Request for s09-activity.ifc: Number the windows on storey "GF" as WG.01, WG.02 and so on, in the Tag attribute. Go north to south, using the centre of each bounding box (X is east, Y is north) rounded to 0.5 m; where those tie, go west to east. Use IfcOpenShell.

First a look at what the model holds.

```python
import ifcopenshell
import ifcopenshell.util.element
import ifcopenshell.util.placement

model = ifcopenshell.open("s09-activity.ifc")
print(model.schema)
storey = next(s for s in model.by_type("IfcBuildingStorey") if s.Name == "GF")
windows = [e for e in ifcopenshell.util.element.get_decomposition(storey) if e.is_a("IfcWindow")]
for e in sorted(windows, key=lambda e: e.id()):
    origin = ifcopenshell.util.placement.get_local_placement(e.ObjectPlacement)[:3, 3]
    print(e.id(), e.Tag, e.Name, origin.round(2) + 0.0, sep=" | ")
```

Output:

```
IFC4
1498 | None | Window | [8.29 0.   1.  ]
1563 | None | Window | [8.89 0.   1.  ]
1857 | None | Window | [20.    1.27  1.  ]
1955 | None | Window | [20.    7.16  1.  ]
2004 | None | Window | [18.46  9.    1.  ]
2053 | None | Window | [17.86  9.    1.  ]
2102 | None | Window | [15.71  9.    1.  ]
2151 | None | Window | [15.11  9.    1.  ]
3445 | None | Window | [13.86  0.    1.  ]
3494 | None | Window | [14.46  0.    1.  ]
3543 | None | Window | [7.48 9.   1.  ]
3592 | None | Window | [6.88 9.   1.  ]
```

```python
import ifcopenshell
import ifcopenshell.geom
import ifcopenshell.util.element
import ifcopenshell.util.shape

model = ifcopenshell.open("s09-activity.ifc")
settings = ifcopenshell.geom.settings()
settings.set("use-world-coords", True)


def centre(element):
    shape = ifcopenshell.geom.create_shape(settings, element)
    return ifcopenshell.util.shape.get_bbox_centroid(shape.geometry)


storey = next(s for s in model.by_type("IfcBuildingStorey") if s.Name == "GF")
windows = [e for e in ifcopenshell.util.element.get_decomposition(storey) if e.is_a("IfcWindow")]

# Insertion points can sit at a corner or the storey origin, so sort by the geometry (in metres).
centres = {e: centre(e) for e in windows}
windows.sort(key=lambda e: (-round(centres[e][1] / 0.5), centres[e][0]))

for i, e in enumerate(windows, start=1):
    number = f"WG.{i:02d}"
    e.Tag = number
    print(e.id(), number)

model.write("s09-activity_v2.ifc")
```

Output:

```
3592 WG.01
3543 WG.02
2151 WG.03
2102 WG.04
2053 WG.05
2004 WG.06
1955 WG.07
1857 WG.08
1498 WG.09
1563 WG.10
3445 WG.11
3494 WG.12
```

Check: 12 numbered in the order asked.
